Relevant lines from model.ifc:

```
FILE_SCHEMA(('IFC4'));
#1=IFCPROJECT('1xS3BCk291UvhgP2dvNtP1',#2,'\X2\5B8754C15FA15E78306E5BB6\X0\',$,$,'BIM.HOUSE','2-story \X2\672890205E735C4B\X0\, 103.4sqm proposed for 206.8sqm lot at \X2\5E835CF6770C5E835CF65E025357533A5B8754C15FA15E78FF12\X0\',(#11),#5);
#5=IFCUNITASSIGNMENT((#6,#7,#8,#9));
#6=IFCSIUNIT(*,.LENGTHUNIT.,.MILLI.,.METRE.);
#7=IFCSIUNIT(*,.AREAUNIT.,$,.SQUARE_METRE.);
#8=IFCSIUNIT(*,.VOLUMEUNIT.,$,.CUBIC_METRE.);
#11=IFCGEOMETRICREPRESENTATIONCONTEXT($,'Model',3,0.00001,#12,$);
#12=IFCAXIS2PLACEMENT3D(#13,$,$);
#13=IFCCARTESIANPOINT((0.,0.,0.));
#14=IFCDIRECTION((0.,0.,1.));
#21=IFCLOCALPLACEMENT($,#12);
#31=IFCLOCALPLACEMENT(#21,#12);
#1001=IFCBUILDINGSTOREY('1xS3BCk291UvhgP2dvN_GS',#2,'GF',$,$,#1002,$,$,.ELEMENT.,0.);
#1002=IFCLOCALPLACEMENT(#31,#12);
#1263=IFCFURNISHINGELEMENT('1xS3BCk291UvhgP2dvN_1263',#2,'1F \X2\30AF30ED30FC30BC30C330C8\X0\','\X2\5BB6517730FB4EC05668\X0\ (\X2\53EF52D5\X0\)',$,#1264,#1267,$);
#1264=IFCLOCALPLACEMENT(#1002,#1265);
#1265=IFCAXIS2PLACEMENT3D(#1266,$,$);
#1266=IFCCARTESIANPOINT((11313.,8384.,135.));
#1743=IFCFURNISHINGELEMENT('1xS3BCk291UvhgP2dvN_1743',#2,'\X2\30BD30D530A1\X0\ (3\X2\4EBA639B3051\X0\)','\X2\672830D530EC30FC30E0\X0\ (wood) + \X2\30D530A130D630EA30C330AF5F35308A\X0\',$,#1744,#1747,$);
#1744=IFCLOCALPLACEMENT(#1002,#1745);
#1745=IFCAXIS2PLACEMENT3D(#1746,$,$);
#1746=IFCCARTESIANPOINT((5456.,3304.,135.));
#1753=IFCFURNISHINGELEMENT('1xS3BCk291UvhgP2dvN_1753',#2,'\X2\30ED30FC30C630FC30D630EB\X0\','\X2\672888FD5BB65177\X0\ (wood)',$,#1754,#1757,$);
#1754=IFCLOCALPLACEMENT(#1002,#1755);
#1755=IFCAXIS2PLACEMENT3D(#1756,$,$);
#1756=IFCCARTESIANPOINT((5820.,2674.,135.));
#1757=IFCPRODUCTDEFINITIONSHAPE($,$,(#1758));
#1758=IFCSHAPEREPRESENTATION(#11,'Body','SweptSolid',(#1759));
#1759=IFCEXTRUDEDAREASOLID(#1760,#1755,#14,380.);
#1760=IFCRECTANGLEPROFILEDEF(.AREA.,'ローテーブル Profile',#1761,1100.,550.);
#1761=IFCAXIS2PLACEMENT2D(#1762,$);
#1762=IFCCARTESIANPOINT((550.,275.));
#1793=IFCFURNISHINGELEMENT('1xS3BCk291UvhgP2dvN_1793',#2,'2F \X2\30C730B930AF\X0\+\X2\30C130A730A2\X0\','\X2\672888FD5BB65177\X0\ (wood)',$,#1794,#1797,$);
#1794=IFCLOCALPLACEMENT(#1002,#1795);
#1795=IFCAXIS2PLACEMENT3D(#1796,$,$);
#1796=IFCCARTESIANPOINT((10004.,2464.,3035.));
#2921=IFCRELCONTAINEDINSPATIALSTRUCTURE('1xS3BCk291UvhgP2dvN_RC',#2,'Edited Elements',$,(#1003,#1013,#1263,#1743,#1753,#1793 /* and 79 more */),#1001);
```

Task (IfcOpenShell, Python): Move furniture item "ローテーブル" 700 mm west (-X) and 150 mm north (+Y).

```python
import ifcopenshell
import ifcopenshell.api.geometry
import ifcopenshell.util.placement
import ifcopenshell.util.unit

model = ifcopenshell.open("model.ifc")
unit_scale = ifcopenshell.util.unit.calculate_unit_scale(model)

item = model.by_guid("1xS3BCk291UvhgP2dvN_1753")
matrix = ifcopenshell.util.placement.get_local_placement(item.ObjectPlacement)
matrix[0, 3] -= 0.7 / unit_scale
matrix[1, 3] += 0.15 / unit_scale
ifcopenshell.api.geometry.edit_object_placement(model, product=item, matrix=matrix, is_si=False)

print(ifcopenshell.util.placement.get_local_placement(item.ObjectPlacement).round(3) + 0.0)

model.write("model_rev.ifc")
```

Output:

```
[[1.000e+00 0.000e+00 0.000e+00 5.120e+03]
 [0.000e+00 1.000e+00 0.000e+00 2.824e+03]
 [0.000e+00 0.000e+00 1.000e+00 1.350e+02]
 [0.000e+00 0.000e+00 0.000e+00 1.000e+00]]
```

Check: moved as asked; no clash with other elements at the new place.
